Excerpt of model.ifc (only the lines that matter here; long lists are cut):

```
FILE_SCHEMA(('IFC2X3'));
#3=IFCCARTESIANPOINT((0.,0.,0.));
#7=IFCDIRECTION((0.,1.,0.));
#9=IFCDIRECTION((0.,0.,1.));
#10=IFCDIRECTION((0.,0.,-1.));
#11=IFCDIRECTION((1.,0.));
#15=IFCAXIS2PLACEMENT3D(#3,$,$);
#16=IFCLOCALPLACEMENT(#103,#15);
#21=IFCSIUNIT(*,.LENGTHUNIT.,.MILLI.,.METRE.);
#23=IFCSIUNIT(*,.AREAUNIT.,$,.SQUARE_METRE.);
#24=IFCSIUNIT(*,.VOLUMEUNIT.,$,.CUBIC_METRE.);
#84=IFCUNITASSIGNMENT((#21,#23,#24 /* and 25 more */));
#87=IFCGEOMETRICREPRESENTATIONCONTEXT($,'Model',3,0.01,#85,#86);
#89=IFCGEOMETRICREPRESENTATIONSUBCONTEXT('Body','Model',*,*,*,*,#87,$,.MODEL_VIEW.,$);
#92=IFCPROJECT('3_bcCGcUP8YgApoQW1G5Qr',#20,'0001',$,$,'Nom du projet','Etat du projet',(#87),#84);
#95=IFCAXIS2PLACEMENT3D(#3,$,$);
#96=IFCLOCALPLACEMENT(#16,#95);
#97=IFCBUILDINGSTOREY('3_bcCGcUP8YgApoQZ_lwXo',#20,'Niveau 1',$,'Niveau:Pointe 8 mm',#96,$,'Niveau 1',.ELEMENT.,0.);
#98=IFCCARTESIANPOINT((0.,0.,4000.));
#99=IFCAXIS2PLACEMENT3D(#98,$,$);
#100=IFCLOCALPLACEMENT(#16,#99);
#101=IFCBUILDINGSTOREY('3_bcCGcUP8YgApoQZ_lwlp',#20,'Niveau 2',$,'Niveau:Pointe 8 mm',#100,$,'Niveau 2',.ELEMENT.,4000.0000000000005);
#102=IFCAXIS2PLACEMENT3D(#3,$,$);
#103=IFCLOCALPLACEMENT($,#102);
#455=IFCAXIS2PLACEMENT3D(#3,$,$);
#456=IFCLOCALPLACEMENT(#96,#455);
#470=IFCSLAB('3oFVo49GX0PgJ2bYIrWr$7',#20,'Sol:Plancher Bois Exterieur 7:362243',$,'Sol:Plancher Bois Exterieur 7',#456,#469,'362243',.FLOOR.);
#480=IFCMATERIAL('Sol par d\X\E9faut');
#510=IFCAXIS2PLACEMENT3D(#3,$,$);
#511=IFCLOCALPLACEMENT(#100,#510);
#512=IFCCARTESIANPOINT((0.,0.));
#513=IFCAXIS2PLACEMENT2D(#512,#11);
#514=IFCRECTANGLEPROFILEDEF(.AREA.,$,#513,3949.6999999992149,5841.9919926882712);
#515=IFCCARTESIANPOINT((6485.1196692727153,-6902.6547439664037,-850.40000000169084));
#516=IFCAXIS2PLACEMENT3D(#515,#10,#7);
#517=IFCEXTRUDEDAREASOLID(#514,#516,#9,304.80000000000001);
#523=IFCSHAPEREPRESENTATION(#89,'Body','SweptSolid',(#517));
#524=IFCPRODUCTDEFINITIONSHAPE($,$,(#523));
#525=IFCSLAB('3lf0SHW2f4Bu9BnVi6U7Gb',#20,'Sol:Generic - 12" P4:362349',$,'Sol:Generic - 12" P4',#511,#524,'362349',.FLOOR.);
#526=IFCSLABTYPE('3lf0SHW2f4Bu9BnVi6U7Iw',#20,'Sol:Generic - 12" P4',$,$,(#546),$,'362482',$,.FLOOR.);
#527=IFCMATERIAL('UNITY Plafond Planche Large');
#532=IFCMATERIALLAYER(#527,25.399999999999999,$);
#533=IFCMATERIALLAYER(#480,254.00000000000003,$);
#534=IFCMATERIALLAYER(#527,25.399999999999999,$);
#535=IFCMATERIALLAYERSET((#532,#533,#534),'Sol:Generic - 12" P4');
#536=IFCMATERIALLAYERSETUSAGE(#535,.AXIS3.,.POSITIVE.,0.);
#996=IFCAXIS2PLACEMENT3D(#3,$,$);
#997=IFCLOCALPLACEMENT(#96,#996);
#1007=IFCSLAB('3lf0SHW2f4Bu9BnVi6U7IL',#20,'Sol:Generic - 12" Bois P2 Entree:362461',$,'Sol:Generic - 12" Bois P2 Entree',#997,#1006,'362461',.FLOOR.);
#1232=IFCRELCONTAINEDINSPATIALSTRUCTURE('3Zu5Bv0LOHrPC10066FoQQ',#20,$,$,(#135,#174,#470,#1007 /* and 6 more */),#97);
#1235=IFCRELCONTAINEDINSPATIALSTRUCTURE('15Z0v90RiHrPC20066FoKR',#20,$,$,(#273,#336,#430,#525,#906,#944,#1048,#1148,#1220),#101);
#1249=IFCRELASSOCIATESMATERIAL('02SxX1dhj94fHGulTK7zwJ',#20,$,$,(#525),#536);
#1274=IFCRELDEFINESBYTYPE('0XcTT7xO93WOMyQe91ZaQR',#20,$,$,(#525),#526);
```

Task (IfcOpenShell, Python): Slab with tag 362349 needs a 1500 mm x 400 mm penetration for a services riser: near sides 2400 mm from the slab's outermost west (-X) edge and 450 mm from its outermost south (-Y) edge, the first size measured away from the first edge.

```python
import numpy as np
import ifcopenshell
import ifcopenshell.api.feature
import ifcopenshell.api.geometry
import ifcopenshell.api.root
import ifcopenshell.geom
import ifcopenshell.util.placement
import ifcopenshell.util.representation
import ifcopenshell.util.shape
import ifcopenshell.util.unit

model = ifcopenshell.open("model.ifc")
unit_scale = ifcopenshell.util.unit.calculate_unit_scale(model)
settings = ifcopenshell.geom.settings()


def volume(element):
    """Net volume in cubic metres, openings subtracted."""
    shape = ifcopenshell.geom.create_shape(settings, element)
    return ifcopenshell.util.shape.get_volume(shape.geometry)


slab = model.by_guid("3lf0SHW2f4Bu9BnVi6U7Gb")
before = volume(slab)

# Extent in the slab's own axes, in metres. The edges named are its -X and -Y sides.
slab_shape = ifcopenshell.geom.create_shape(settings, slab)
vertices = ifcopenshell.util.shape.get_vertices(slab_shape.geometry)
x_min, y_min, bottom = vertices.min(axis=0)
top = vertices[:, 2].max()

opening = ifcopenshell.api.root.create_entity(model, ifc_class="IfcOpeningElement", name="Services riser opening")
context = ifcopenshell.util.representation.get_context(model, "Model", "Body", "MODEL_VIEW")
width, depth = 1.5, 0.4
outline = [(0.0, 0.0), (width, 0.0), (width, depth), (0.0, depth), (0.0, 0.0)]
# Overshoot both faces by 50 mm so the cut is clean.
shape = ifcopenshell.api.geometry.add_slab_representation(
    model, context=context, depth=top - bottom + 0.1, polyline=outline
)
ifcopenshell.api.geometry.assign_representation(model, product=opening, representation=shape)

matrix = ifcopenshell.util.placement.get_local_placement(slab.ObjectPlacement)
matrix[:, 3] = matrix @ np.append(np.array([x_min + 2.4, y_min + 0.45, bottom - 0.05]) / unit_scale, 1.0)
ifcopenshell.api.geometry.edit_object_placement(model, product=opening, matrix=matrix, is_si=False)
ifcopenshell.api.feature.add_feature(model, feature=opening, element=slab)

after = volume(slab)

print(f"slab volume {before:.3f} -> {after:.3f} m3")

model.write("model_rev.ifc")
```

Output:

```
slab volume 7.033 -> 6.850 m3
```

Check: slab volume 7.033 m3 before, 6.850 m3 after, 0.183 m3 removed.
